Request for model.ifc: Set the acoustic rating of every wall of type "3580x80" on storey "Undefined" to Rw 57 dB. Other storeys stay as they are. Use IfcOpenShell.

First a look at what the model holds.

```python
import ifcopenshell
import ifcopenshell.util.element

model = ifcopenshell.open("model.ifc")
print(model.schema)
storey = next(s for s in model.by_type("IfcBuildingStorey") if s.Name == "Undefined")
walls = [e for e in ifcopenshell.util.element.get_decomposition(storey) if e.is_a("IfcWall")]
seen = {}
for e in walls:
    element_type = ifcopenshell.util.element.get_type(e)
    key = (element_type.Name if element_type != e and element_type else None, ifcopenshell.util.element.get_pset(e, "Pset_WallCommon", "AcousticRating"))
    seen[key] = seen.get(key, 0) + 1
for (name, value), count in sorted(seen.items(), key=str):
    print(count, "x", name, "|", value)
```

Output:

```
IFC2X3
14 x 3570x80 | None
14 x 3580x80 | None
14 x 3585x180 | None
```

```python
import ifcopenshell
import ifcopenshell.api.pset
import ifcopenshell.util.element

model = ifcopenshell.open("model.ifc")

storey = next(s for s in model.by_type("IfcBuildingStorey") if s.Name == "Undefined")
walls = [e for e in ifcopenshell.util.element.get_decomposition(storey) if e.is_a("IfcWall")]

count = 0
for e in walls:
    element_type = ifcopenshell.util.element.get_type(e)
    if element_type in (None, e) or element_type.Name != "3580x80":
        continue
    found = ifcopenshell.util.element.get_pset(e, "Pset_WallCommon", should_inherit=False)
    if found:
        pset = model.by_id(found["id"])
        if len(ifcopenshell.util.element.get_elements_by_pset(pset)) > 1:
            pset = ifcopenshell.api.pset.unshare_pset(model, products=[e], pset=pset)[0]
    else:
        pset = ifcopenshell.api.pset.add_pset(model, product=e, name="Pset_WallCommon")
    ifcopenshell.api.pset.edit_pset(model, pset=pset, properties={"AcousticRating": "Rw 57 dB"})
    count += 1

print(count, "walls updated")

model.write("model_updated.ifc")
```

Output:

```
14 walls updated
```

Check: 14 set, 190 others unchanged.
